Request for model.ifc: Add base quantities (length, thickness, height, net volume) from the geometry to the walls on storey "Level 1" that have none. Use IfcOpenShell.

First a look at what the model holds.

```python
import ifcopenshell
import ifcopenshell.util.element
import ifcopenshell.util.unit

model = ifcopenshell.open("model.ifc")
print(model.schema)
for unit_type in ("LENGTHUNIT", "AREAUNIT", "VOLUMEUNIT"):
    print(unit_type, ifcopenshell.util.unit.calculate_unit_scale(model, unit_type))
storey = next(s for s in model.by_type("IfcBuildingStorey") if s.Name == "Level 1")
walls = [e for e in ifcopenshell.util.element.get_decomposition(storey) if e.is_a("IfcWall")]
for e in sorted(walls, key=lambda e: e.id()):
    print(e.id(), e.is_a(), e.Name, list(ifcopenshell.util.element.get_psets(e, qtos_only=True)), sep=" | ")
```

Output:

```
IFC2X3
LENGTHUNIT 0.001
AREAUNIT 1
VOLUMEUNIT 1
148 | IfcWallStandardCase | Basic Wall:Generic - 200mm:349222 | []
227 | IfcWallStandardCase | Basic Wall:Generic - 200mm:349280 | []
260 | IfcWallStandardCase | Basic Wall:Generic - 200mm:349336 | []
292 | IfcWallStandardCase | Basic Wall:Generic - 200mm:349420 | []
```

```python
import ifcopenshell
import ifcopenshell.api.pset
import ifcopenshell.geom
import ifcopenshell.util.element
import ifcopenshell.util.shape
import ifcopenshell.util.unit

model = ifcopenshell.open("model.ifc")
unit_scale = ifcopenshell.util.unit.calculate_unit_scale(model)
volume_scale = ifcopenshell.util.unit.calculate_unit_scale(model, "VOLUMEUNIT")
settings = ifcopenshell.geom.settings()

storey = next(s for s in model.by_type("IfcBuildingStorey") if s.Name == "Level 1")
walls = [e for e in ifcopenshell.util.element.get_decomposition(storey) if e.is_a("IfcWall")]

for e in sorted(walls, key=lambda e: e.id()):
    if ifcopenshell.util.element.get_psets(e, qtos_only=True, should_inherit=False):
        continue
    # Geometry comes back in metres, in the element's own axes.
    shape = ifcopenshell.geom.create_shape(settings, e)
    values = {
        "Length": ifcopenshell.util.shape.get_x(shape.geometry) / unit_scale,
        "Width": ifcopenshell.util.shape.get_y(shape.geometry) / unit_scale,
        "Height": ifcopenshell.util.shape.get_z(shape.geometry) / unit_scale,
        "NetVolume": ifcopenshell.util.shape.get_volume(shape.geometry) / volume_scale,
    }
    qto = ifcopenshell.api.pset.add_qto(model, product=e, name="BaseQuantities")
    ifcopenshell.api.pset.edit_qto(model, qto=qto, properties=values)
    print(e.id(), {k: round(v, 3) for k, v in values.items()})

model.write("model_updated.ifc")
```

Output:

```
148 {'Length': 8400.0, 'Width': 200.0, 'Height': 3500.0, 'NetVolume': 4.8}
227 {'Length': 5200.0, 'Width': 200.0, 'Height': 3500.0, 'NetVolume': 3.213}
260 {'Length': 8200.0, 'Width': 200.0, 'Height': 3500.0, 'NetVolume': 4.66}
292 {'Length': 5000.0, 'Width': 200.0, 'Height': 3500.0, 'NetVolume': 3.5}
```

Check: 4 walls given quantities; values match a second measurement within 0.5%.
